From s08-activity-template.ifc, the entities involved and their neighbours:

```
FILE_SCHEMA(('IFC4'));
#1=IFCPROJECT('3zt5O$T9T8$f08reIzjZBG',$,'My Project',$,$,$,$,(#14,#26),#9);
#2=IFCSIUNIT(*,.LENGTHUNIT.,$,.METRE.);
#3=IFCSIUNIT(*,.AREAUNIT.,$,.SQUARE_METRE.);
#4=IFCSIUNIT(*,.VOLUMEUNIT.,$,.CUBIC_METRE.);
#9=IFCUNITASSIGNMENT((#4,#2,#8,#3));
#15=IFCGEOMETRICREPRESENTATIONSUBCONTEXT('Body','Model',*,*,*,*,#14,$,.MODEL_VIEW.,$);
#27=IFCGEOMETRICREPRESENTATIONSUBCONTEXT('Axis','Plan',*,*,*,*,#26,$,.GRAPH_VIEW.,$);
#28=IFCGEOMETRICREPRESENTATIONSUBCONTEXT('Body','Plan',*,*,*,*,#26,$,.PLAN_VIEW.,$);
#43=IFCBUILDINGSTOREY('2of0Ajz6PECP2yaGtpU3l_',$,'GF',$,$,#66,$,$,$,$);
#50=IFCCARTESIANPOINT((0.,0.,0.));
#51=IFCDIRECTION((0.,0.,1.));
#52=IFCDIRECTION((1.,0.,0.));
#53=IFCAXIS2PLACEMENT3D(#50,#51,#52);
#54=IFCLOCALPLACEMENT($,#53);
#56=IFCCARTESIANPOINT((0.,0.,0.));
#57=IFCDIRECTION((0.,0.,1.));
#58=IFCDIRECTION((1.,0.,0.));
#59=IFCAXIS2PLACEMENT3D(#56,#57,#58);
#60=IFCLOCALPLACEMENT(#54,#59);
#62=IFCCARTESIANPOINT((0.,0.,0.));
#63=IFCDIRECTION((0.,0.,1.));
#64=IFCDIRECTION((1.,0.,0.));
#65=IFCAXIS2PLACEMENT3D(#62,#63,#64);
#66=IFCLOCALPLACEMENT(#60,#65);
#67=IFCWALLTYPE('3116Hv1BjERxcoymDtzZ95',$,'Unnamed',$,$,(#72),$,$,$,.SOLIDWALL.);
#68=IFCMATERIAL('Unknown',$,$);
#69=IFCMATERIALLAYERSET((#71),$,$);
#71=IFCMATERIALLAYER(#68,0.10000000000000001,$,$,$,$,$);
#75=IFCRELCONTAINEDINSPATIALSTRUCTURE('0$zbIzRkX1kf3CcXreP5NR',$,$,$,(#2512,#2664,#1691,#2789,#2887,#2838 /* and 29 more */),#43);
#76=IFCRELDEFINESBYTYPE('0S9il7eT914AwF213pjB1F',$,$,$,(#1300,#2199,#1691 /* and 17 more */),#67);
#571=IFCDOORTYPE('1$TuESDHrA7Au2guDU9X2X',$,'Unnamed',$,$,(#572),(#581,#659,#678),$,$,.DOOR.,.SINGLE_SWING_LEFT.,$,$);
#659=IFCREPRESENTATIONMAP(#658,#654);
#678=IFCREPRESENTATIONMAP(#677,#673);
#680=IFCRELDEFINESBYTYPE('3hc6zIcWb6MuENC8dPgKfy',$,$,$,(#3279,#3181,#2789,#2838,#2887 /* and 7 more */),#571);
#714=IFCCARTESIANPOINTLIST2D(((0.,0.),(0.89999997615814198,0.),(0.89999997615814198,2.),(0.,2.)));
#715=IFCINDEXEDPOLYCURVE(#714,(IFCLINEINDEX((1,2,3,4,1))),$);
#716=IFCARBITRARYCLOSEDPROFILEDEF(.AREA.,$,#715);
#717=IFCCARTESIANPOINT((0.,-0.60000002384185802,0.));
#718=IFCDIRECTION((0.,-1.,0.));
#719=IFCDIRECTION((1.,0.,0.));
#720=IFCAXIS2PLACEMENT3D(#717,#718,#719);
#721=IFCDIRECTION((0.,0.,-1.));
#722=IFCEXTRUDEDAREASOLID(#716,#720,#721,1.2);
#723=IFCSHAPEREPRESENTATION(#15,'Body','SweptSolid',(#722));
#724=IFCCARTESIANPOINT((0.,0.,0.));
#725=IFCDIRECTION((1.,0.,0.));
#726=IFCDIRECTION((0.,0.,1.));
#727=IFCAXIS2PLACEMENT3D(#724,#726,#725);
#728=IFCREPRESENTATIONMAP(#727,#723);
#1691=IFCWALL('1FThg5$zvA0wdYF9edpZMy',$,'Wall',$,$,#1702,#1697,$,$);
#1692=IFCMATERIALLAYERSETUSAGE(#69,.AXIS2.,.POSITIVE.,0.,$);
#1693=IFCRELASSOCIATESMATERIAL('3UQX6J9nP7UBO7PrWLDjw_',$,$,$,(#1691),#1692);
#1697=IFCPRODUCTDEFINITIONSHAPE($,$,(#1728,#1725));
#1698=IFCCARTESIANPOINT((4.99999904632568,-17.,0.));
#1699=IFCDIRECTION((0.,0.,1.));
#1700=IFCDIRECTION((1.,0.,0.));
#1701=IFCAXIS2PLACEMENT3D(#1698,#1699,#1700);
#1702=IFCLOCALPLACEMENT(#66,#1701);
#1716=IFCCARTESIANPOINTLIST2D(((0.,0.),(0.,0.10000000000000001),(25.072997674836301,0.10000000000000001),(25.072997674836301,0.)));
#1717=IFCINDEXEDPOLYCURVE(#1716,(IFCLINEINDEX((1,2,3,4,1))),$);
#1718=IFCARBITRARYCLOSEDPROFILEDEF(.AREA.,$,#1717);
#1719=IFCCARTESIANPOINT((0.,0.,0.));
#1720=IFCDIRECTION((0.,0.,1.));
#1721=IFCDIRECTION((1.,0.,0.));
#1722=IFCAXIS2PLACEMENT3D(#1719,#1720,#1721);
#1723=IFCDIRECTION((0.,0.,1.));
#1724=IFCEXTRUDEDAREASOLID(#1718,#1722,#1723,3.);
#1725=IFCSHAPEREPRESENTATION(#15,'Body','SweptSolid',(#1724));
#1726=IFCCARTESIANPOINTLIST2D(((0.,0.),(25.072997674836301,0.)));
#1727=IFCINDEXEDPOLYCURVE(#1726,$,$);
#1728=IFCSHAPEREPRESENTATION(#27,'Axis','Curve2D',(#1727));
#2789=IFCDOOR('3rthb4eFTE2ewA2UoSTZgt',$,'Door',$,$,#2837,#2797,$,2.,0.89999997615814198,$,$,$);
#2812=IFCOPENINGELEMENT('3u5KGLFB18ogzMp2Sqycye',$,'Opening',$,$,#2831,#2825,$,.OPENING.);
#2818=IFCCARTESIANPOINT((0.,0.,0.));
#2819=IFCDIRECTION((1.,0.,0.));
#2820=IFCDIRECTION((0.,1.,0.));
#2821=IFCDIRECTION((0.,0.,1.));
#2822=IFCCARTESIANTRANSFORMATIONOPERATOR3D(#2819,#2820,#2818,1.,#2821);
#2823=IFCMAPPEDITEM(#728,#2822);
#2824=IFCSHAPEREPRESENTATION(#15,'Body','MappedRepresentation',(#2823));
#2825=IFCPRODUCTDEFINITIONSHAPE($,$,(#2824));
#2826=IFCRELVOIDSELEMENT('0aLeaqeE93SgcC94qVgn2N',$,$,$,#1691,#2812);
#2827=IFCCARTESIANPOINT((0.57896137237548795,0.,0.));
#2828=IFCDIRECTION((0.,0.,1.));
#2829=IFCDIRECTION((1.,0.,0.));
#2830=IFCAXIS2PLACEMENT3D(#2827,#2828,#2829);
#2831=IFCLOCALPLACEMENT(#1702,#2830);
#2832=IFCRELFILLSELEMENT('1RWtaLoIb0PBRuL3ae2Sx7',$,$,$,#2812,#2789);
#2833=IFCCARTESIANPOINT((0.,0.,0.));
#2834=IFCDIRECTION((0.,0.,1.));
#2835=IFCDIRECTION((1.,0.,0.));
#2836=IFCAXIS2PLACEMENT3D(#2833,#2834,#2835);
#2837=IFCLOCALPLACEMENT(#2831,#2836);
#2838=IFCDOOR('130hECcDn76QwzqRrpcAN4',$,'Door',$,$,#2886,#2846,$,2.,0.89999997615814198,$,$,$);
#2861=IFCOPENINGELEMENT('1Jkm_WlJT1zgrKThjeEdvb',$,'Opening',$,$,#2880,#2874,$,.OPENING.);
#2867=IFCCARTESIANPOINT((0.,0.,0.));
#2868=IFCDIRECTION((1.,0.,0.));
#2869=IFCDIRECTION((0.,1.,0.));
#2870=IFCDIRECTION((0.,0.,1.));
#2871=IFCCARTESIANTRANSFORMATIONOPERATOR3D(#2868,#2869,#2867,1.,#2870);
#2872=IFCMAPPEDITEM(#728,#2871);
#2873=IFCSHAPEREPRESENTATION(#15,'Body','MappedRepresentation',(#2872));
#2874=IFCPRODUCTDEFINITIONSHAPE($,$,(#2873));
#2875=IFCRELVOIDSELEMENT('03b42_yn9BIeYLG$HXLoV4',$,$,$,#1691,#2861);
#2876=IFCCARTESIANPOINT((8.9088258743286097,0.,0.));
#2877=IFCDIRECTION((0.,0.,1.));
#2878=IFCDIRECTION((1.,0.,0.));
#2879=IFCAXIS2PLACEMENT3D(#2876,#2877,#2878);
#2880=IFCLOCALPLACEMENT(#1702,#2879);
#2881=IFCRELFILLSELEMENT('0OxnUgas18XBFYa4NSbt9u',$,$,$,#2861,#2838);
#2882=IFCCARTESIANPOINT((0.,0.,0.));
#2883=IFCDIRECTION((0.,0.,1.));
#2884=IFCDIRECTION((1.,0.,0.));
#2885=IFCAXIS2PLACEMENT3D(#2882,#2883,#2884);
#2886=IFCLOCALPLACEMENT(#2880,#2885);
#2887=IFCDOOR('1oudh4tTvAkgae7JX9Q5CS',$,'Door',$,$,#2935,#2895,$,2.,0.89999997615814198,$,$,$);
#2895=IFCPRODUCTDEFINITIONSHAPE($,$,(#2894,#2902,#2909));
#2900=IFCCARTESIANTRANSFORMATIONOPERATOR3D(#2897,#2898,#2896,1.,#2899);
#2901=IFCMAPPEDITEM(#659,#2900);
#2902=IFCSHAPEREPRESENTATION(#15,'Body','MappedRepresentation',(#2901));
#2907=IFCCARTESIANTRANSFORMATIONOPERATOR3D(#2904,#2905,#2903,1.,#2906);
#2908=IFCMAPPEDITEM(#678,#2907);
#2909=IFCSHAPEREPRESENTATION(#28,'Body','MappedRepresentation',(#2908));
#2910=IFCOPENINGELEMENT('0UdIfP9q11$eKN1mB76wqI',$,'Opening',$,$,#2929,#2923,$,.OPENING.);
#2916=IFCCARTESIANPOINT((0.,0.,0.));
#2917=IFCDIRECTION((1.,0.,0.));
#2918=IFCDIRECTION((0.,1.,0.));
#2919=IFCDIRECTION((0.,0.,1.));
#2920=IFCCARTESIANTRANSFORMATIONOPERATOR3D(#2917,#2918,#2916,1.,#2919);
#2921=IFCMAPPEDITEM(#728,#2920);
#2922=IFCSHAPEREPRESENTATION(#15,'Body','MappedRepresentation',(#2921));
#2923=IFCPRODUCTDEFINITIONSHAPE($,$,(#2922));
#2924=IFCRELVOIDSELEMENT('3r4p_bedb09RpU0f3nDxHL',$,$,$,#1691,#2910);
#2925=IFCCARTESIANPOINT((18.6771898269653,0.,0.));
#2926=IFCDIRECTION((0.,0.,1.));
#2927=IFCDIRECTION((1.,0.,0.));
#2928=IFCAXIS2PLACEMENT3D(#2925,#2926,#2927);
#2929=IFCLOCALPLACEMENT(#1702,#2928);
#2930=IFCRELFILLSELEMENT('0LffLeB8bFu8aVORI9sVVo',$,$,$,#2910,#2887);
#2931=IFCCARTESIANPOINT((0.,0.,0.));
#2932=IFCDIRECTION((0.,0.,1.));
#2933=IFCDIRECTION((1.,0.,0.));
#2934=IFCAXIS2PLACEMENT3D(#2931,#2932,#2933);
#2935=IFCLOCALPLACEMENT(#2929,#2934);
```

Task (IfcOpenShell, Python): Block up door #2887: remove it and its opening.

```python
import ifcopenshell
import ifcopenshell.api.feature
import ifcopenshell.api.root
import ifcopenshell.geom
import ifcopenshell.util.shape

model = ifcopenshell.open("s08-activity-template.ifc")
settings = ifcopenshell.geom.settings()


def volume(element):
    """Net volume in cubic metres, openings subtracted."""
    shape = ifcopenshell.geom.create_shape(settings, element)
    return ifcopenshell.util.shape.get_volume(shape.geometry)


door = model.by_guid("1oudh4tTvAkgae7JX9Q5CS")
opening = door.FillsVoids[0].RelatingOpeningElement
wall = opening.VoidsElements[0].RelatingBuildingElement
before = volume(wall)

ifcopenshell.api.root.remove_product(model, product=door)
ifcopenshell.api.feature.remove_feature(model, feature=opening)

after = volume(wall)

print(f"wall volume {before:.3f} -> {after:.3f} m3")

model.write("s08-activity-template_v2.ifc")
```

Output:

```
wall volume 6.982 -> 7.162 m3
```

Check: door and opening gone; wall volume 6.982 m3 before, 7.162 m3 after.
